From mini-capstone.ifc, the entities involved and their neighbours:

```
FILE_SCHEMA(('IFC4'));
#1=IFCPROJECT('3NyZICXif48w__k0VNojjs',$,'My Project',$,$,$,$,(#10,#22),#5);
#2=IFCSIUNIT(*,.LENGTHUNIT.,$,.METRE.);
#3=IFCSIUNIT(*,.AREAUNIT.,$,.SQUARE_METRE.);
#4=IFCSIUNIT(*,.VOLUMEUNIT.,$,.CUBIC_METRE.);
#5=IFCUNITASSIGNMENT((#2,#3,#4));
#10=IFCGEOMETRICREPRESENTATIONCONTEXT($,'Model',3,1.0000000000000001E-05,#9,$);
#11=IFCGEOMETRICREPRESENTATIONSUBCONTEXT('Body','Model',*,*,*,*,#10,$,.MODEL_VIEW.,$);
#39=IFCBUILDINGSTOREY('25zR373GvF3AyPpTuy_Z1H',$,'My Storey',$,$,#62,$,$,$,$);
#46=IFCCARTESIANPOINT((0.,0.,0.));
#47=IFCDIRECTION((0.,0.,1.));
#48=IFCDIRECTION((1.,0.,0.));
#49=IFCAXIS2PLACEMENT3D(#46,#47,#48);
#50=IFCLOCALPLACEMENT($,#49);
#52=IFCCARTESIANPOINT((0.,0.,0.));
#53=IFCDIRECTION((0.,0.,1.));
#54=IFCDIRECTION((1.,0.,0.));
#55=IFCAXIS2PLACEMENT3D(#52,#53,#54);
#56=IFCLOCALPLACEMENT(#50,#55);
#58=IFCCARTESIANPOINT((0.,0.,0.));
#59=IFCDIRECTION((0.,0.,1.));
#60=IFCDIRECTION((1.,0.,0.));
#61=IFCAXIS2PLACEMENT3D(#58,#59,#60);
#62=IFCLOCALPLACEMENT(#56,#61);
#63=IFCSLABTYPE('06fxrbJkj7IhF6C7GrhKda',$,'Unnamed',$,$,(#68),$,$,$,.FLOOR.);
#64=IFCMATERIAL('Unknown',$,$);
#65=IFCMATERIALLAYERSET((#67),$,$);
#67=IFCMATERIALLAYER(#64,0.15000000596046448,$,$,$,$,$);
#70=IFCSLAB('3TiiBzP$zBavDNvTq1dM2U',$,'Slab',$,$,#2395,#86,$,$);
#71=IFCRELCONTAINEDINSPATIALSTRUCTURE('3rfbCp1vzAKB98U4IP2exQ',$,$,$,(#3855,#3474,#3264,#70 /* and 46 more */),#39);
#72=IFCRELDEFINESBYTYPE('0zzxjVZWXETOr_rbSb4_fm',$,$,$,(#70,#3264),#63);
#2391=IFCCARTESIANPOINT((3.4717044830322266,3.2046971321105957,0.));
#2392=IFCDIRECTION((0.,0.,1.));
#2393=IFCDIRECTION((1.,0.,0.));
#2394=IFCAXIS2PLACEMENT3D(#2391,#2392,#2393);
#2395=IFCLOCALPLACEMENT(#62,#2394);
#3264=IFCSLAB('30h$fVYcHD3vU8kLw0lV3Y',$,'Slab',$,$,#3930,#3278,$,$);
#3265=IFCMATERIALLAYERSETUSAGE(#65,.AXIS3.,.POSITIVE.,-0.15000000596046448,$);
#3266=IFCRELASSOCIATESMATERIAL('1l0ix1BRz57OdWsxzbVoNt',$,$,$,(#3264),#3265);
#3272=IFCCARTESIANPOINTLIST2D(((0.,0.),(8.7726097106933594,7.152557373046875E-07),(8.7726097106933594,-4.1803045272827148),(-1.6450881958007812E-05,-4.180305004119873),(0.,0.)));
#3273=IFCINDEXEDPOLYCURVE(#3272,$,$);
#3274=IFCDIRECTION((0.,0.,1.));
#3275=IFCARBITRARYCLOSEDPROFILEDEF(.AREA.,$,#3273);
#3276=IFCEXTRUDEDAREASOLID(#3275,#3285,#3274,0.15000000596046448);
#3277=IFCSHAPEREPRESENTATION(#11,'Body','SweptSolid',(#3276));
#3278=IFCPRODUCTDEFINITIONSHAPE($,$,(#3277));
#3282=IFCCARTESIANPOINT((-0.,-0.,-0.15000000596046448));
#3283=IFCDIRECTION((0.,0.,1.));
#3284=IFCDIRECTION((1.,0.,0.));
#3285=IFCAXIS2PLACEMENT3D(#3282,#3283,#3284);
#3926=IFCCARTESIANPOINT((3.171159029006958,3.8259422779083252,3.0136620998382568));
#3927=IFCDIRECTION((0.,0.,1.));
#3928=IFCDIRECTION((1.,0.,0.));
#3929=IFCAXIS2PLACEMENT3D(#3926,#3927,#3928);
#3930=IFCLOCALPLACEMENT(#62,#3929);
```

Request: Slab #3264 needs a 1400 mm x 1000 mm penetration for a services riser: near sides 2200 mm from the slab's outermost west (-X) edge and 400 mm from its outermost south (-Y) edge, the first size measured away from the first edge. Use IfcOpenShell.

```python
import numpy as np
import ifcopenshell
import ifcopenshell.api.feature
import ifcopenshell.api.geometry
import ifcopenshell.api.root
import ifcopenshell.geom
import ifcopenshell.util.placement
import ifcopenshell.util.representation
import ifcopenshell.util.shape
import ifcopenshell.util.unit

model = ifcopenshell.open("mini-capstone.ifc")
unit_scale = ifcopenshell.util.unit.calculate_unit_scale(model)
settings = ifcopenshell.geom.settings()


def volume(element):
    """Net volume in cubic metres, openings subtracted."""
    shape = ifcopenshell.geom.create_shape(settings, element)
    return ifcopenshell.util.shape.get_volume(shape.geometry)


slab = model.by_guid("30h$fVYcHD3vU8kLw0lV3Y")
before = volume(slab)

# Extent in the slab's own axes, in metres. The edges named are its -X and -Y sides.
slab_shape = ifcopenshell.geom.create_shape(settings, slab)
vertices = ifcopenshell.util.shape.get_vertices(slab_shape.geometry)
x_min, y_min, bottom = vertices.min(axis=0)
top = vertices[:, 2].max()

opening = ifcopenshell.api.root.create_entity(model, ifc_class="IfcOpeningElement", name="Services riser opening", predefined_type="OPENING")
context = ifcopenshell.util.representation.get_context(model, "Model", "Body", "MODEL_VIEW")
width, depth = 1.4, 1
outline = [(0.0, 0.0), (width, 0.0), (width, depth), (0.0, depth), (0.0, 0.0)]
# Overshoot both faces by 50 mm so the cut is clean.
shape = ifcopenshell.api.geometry.add_slab_representation(
    model, context=context, depth=top - bottom + 0.1, polyline=outline
)
ifcopenshell.api.geometry.assign_representation(model, product=opening, representation=shape)

matrix = ifcopenshell.util.placement.get_local_placement(slab.ObjectPlacement)
matrix[:, 3] = matrix @ np.append(np.array([x_min + 2.2, y_min + 0.4, bottom - 0.05]) / unit_scale, 1.0)
ifcopenshell.api.geometry.edit_object_placement(model, product=opening, matrix=matrix, is_si=False)
ifcopenshell.api.feature.add_feature(model, feature=opening, element=slab)

after = volume(slab)

print(f"slab volume {before:.3f} -> {after:.3f} m3")

model.write("mini-capstone-out.ifc")
```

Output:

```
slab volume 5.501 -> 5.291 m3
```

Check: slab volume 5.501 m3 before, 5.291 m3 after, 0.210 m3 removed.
